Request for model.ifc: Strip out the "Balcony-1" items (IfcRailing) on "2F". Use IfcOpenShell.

First a look at what the model holds.

```python
import ifcopenshell
import ifcopenshell.util.element

model = ifcopenshell.open("model.ifc")
print(model.schema)
storey = next(s for s in model.by_type("IfcBuildingStorey") if s.Name == "2F")
railings = [e for e in ifcopenshell.util.element.get_decomposition(storey) if e.is_a("IfcRailing")]
seen = {}
for e in railings:
    element_type = ifcopenshell.util.element.get_type(e)
    name = element_type.Name if element_type not in (None, e) else None
    seen[name] = seen.get(name, 0) + 1
for name, count in sorted(seen.items(), key=str):
    print(count, "x", name)
```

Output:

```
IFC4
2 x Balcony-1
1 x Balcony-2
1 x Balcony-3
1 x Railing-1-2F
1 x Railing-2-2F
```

```python
import ifcopenshell
import ifcopenshell.api.root
import ifcopenshell.util.element

model = ifcopenshell.open("model.ifc")

storey = next(s for s in model.by_type("IfcBuildingStorey") if s.Name == "2F")
railings = [e for e in ifcopenshell.util.element.get_decomposition(storey) if e.is_a("IfcRailing")]
targets = [e for e in railings if (t := ifcopenshell.util.element.get_type(e)) not in (None, e) and t.Name == "Balcony-1"]

for e in targets:
    ifcopenshell.api.root.remove_product(model, product=e)
print(len(targets), "removed")

model.write("model_edited.ifc")
```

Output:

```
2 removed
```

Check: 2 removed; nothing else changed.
